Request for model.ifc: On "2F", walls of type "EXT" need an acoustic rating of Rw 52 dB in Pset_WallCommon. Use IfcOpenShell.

First a look at what the model holds.

```python
import ifcopenshell
import ifcopenshell.util.element

model = ifcopenshell.open("model.ifc")
print(model.schema)
storey = next(s for s in model.by_type("IfcBuildingStorey") if s.Name == "2F")
walls = [e for e in ifcopenshell.util.element.get_decomposition(storey) if e.is_a("IfcWall")]
seen = {}
for e in walls:
    element_type = ifcopenshell.util.element.get_type(e)
    key = (element_type.Name if element_type != e and element_type else None, ifcopenshell.util.element.get_pset(e, "Pset_WallCommon", "AcousticRating"))
    seen[key] = seen.get(key, 0) + 1
for (name, value), count in sorted(seen.items(), key=str):
    print(count, "x", name, "|", value)
```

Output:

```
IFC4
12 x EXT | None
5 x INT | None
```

```python
import ifcopenshell
import ifcopenshell.api.pset
import ifcopenshell.util.element

model = ifcopenshell.open("model.ifc")

storey = next(s for s in model.by_type("IfcBuildingStorey") if s.Name == "2F")
walls = [e for e in ifcopenshell.util.element.get_decomposition(storey) if e.is_a("IfcWall")]

count = 0
for e in walls:
    element_type = ifcopenshell.util.element.get_type(e)
    if element_type in (None, e) or element_type.Name != "EXT":
        continue
    # add_pset returns the element's existing set when there is one.
    pset = ifcopenshell.api.pset.add_pset(model, product=e, name="Pset_WallCommon")
    ifcopenshell.api.pset.edit_pset(model, pset=pset, properties={"AcousticRating": "Rw 52 dB"})
    count += 1

print(count, "walls updated")

model.write("model_updated.ifc")
```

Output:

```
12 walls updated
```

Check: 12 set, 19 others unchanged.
